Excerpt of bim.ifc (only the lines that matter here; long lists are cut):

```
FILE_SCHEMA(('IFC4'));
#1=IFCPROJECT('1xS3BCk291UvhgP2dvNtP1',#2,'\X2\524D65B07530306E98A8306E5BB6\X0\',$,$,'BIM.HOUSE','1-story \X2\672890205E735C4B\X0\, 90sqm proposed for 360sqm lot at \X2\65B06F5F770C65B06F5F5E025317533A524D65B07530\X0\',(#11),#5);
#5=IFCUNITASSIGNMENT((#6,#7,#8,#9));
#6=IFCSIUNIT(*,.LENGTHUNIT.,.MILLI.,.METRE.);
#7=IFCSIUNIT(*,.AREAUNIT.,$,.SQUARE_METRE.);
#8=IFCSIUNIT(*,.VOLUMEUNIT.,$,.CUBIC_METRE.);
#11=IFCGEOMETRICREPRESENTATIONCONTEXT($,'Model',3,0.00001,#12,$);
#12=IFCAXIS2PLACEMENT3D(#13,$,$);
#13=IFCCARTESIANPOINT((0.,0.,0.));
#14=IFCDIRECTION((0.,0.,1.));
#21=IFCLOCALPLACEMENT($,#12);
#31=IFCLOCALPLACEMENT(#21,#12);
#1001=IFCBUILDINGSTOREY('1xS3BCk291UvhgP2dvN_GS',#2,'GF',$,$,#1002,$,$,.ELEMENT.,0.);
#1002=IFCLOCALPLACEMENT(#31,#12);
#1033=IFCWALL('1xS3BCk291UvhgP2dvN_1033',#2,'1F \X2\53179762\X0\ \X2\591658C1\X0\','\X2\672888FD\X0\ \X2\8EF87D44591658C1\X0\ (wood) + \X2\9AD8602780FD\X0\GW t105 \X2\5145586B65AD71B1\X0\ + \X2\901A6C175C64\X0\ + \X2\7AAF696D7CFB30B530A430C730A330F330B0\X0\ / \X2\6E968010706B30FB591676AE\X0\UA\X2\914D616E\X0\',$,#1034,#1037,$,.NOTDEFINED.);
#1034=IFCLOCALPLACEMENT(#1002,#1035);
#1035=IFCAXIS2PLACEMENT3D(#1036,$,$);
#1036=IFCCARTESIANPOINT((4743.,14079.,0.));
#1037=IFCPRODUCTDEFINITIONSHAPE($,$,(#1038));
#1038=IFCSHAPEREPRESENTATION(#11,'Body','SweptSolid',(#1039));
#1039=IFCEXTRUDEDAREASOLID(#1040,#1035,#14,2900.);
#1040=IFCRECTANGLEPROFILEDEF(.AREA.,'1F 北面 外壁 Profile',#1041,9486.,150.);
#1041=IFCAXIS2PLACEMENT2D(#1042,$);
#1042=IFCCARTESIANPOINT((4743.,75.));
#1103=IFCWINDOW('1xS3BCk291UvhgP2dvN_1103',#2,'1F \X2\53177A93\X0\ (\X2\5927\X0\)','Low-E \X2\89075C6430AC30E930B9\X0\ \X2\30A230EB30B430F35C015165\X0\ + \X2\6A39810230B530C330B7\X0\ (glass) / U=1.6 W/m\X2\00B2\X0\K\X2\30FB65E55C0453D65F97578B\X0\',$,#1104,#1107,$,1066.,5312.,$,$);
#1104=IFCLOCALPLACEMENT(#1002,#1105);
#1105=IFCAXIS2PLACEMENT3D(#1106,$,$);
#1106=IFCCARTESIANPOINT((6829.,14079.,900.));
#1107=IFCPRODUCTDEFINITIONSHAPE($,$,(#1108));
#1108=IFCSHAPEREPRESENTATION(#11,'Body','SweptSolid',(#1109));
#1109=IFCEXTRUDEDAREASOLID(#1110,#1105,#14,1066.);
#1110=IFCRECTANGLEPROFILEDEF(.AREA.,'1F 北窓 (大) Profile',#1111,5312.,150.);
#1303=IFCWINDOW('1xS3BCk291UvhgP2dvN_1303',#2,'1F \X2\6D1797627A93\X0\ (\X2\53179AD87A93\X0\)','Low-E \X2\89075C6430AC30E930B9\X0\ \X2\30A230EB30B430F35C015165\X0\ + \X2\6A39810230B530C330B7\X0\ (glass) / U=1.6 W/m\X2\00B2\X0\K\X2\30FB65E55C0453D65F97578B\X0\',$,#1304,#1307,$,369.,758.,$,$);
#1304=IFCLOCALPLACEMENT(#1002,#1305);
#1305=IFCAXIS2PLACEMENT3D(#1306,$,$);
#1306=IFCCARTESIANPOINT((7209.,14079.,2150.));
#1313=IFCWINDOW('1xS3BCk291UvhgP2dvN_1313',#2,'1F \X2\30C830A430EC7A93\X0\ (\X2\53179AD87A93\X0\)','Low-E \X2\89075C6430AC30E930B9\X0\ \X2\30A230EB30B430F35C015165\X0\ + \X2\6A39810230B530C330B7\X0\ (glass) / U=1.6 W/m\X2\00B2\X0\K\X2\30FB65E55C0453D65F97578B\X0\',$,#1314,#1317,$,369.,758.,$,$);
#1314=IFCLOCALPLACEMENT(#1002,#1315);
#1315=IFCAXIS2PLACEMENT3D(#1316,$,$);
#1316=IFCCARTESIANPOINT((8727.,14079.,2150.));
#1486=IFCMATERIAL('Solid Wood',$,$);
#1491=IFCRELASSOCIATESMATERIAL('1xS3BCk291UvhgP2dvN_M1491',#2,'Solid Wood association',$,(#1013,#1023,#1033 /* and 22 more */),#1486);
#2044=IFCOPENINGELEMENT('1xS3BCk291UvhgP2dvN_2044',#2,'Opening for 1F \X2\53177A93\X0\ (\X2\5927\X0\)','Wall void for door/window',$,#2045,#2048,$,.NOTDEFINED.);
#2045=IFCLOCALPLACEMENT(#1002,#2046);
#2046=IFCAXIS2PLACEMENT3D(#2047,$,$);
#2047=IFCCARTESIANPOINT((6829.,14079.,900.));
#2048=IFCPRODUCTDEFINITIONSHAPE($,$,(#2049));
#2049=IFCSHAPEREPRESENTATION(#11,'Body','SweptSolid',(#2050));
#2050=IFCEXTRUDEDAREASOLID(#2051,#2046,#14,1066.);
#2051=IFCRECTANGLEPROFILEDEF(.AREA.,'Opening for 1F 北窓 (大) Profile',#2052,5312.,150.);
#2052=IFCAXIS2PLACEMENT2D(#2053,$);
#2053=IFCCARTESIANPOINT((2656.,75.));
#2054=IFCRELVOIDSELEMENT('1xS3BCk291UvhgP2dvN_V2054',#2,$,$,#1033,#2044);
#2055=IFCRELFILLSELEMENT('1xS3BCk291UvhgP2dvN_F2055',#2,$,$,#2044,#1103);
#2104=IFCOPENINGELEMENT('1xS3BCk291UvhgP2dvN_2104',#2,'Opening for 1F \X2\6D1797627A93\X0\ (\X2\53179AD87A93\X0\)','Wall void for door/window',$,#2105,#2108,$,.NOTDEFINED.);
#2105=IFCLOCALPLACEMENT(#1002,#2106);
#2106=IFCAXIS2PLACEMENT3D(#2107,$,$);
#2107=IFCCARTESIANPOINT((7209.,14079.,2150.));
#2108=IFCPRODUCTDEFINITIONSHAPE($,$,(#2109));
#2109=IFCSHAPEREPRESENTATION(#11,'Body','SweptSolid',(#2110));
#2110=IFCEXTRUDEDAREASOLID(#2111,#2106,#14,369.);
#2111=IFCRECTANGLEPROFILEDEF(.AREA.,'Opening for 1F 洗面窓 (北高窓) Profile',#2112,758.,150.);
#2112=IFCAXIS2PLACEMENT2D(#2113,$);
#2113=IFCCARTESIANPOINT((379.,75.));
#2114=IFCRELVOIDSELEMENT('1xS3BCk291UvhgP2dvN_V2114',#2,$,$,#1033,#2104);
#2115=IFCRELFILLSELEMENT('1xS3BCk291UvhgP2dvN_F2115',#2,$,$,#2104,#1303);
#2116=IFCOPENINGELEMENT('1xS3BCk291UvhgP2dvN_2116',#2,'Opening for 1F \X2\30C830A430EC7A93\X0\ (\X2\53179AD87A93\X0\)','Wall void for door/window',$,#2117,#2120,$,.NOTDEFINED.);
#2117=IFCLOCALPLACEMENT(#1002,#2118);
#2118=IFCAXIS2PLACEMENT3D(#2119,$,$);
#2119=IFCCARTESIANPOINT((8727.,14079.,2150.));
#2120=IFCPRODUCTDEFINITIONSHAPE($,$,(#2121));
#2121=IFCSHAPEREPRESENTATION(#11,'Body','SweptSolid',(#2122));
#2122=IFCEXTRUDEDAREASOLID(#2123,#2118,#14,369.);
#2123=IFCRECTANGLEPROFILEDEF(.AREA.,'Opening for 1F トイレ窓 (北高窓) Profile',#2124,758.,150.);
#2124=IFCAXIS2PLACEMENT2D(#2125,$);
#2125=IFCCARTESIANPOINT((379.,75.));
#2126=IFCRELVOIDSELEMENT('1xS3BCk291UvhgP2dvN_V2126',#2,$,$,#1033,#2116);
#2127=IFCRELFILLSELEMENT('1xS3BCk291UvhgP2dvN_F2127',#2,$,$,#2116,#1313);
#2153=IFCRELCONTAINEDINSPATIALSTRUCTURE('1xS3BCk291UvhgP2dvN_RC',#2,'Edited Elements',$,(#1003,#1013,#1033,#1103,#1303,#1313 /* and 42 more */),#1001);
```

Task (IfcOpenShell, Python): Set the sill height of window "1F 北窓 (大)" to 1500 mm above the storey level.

```python
import numpy as np
import ifcopenshell
import ifcopenshell.api.geometry
import ifcopenshell.geom
import ifcopenshell.util.element
import ifcopenshell.util.placement
import ifcopenshell.util.shape
import ifcopenshell.util.unit

model = ifcopenshell.open("bim.ifc")
unit_scale = ifcopenshell.util.unit.calculate_unit_scale(model)

window = model.by_guid("1xS3BCk291UvhgP2dvN_1103")
opening = window.FillsVoids[0].RelatingOpeningElement
storey = ifcopenshell.util.element.get_container(window, ifc_class="IfcBuildingStorey")
level = ifcopenshell.util.placement.get_local_placement(storey.ObjectPlacement)[2, 3]

# The opening's origin need not be at the sill, so measure its lowest point.
shape = ifcopenshell.geom.create_shape(ifcopenshell.geom.settings(), opening)
bottom = ifcopenshell.util.shape.get_shape_bottom_elevation(shape, shape.geometry) / unit_scale
dz = level + 1.5 / unit_scale - bottom

shift = np.array([0.0, 0.0, dz])
# The window is not placed relative to its opening, so move both.
for product in (opening, window):
    matrix = ifcopenshell.util.placement.get_local_placement(product.ObjectPlacement)
    matrix[:3, 3] += shift
    ifcopenshell.api.geometry.edit_object_placement(model, product=product, matrix=matrix, is_si=False)

print(f"moved by {dz * unit_scale:+.3f} m")

model.write("bim_v2.ifc")
```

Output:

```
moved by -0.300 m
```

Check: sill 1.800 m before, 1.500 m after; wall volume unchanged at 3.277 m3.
